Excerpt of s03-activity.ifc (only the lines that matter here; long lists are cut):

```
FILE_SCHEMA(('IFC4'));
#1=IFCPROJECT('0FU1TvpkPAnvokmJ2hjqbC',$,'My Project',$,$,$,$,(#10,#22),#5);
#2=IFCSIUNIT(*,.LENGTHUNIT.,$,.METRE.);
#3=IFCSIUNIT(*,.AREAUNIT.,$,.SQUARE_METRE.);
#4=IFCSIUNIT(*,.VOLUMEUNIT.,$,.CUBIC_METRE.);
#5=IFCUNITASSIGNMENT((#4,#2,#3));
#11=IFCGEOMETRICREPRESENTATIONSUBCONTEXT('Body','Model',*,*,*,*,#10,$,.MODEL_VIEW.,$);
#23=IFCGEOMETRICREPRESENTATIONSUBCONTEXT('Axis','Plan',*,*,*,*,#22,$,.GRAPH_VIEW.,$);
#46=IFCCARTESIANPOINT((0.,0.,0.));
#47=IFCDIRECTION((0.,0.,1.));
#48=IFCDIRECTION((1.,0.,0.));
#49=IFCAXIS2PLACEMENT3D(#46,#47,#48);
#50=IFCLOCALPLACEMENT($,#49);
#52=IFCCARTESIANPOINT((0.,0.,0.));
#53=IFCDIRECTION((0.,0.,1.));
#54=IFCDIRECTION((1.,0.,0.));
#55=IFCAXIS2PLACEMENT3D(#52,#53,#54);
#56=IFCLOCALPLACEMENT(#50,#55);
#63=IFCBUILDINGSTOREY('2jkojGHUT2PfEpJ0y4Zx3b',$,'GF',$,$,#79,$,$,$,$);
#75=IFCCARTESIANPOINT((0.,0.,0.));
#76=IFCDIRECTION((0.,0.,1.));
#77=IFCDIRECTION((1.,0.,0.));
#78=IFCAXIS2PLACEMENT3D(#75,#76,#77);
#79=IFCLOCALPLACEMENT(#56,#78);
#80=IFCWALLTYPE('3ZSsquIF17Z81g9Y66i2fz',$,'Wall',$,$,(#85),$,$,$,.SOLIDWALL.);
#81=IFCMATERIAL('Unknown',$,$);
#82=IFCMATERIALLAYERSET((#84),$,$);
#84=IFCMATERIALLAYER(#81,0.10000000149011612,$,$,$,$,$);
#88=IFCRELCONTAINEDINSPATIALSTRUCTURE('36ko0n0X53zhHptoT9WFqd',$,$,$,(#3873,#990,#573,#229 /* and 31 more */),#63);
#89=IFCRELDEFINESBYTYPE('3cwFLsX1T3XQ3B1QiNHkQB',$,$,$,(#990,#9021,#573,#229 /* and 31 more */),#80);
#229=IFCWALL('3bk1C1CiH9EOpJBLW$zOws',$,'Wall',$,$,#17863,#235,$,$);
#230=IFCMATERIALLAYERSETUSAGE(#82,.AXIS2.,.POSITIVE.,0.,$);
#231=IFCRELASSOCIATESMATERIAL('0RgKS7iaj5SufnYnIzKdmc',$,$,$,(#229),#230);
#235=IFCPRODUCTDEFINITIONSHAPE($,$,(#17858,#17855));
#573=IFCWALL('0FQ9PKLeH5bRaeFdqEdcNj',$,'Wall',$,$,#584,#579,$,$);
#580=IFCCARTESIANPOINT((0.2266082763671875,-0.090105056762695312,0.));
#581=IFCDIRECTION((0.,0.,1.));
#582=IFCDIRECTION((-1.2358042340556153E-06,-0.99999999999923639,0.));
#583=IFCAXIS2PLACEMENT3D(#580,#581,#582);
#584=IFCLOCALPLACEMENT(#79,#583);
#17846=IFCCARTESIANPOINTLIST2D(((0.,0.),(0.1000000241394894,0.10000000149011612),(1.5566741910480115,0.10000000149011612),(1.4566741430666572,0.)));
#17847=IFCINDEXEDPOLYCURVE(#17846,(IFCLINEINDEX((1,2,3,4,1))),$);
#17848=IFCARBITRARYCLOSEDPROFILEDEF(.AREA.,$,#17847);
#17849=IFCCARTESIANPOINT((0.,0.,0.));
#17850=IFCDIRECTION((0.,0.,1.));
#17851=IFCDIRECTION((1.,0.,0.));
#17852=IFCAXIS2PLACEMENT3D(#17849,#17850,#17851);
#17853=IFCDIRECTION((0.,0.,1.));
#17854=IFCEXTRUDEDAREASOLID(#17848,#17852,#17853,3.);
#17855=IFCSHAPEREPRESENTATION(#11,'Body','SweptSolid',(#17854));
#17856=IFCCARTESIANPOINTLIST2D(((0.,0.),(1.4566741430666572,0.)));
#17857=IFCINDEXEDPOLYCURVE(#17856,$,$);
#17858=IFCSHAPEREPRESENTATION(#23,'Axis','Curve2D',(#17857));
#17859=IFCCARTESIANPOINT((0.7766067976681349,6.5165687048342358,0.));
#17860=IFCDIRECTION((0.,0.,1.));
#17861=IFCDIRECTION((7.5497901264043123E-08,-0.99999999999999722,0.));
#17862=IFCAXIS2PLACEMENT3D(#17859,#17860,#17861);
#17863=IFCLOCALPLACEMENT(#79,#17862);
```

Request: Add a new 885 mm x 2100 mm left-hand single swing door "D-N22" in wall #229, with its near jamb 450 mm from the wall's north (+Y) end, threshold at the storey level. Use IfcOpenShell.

```python
import numpy as np
import ifcopenshell
import ifcopenshell.api.feature
import ifcopenshell.api.geometry
import ifcopenshell.api.root
import ifcopenshell.api.spatial
import ifcopenshell.geom
import ifcopenshell.util.element
import ifcopenshell.util.placement
import ifcopenshell.util.representation
import ifcopenshell.util.shape
import ifcopenshell.util.unit

model = ifcopenshell.open("s03-activity.ifc")
unit_scale = ifcopenshell.util.unit.calculate_unit_scale(model)
settings = ifcopenshell.geom.settings()


def volume(element):
    """Net volume in cubic metres, openings subtracted."""
    shape = ifcopenshell.geom.create_shape(settings, element)
    return ifcopenshell.util.shape.get_volume(shape.geometry)


wall = model.by_id(229)
storey = ifcopenshell.util.element.get_container(wall, ifc_class="IfcBuildingStorey")
context = ifcopenshell.util.representation.get_context(model, "Model", "Body", "MODEL_VIEW")
before = volume(wall)

width, height, from_end, sill = 0.885, 2.1, 0.45, 0.0  # metres

# The wall runs along its own X axis, and the end named is its -X end.
wall_shape = ifcopenshell.geom.create_shape(settings, wall)
x, y, z = ifcopenshell.util.shape.get_vertices(wall_shape.geometry).T
start = x.min() + from_end
face, thickness = float(y.min()), float(y.max() - y.min())
wall_matrix = ifcopenshell.util.placement.get_local_placement(wall.ObjectPlacement)
level = ifcopenshell.util.placement.get_local_placement(storey.ObjectPlacement)[2, 3]


def in_wall(x, y):
    """Placement at x, y metres in the wall's axes, at sill height."""
    matrix = wall_matrix.copy()
    matrix[:, 3] = wall_matrix @ np.array([x / unit_scale, y / unit_scale, 0.0, 1.0])
    matrix[2, 3] = level + sill / unit_scale
    return matrix


# Opening: a box that overshoots both wall faces by 50 mm.
opening = ifcopenshell.api.root.create_entity(model, ifc_class="IfcOpeningElement", predefined_type="OPENING")
box = ifcopenshell.api.geometry.add_wall_representation(
    model, context=context, length=width, height=height, thickness=thickness + 0.1
)
ifcopenshell.api.geometry.assign_representation(model, product=opening, representation=box)
ifcopenshell.api.geometry.edit_object_placement(model, product=opening, matrix=in_wall(start, face - 0.05), is_si=False)
ifcopenshell.api.feature.add_feature(model, feature=opening, element=wall)

door = ifcopenshell.api.root.create_entity(model, ifc_class="IfcDoor", name="D-N22", predefined_type="DOOR")
door.OverallWidth, door.OverallHeight = width / unit_scale, height / unit_scale
door.OperationType = "SINGLE_SWING_LEFT"
body = ifcopenshell.api.geometry.add_door_representation(
    model,
    context=context,
    overall_width=door.OverallWidth,
    overall_height=door.OverallHeight,
    operation_type="SINGLE_SWING_LEFT",
    lining_properties={"LiningDepth": thickness / unit_scale, "ThresholdDepth": thickness / unit_scale},
)
ifcopenshell.api.geometry.assign_representation(model, product=door, representation=body)
ifcopenshell.api.spatial.assign_container(model, products=[door], relating_structure=storey)
ifcopenshell.api.feature.add_filling(model, opening=opening, element=door)

# The lining spans the wall, so the door starts at the wall face.
ifcopenshell.api.geometry.edit_object_placement(model, product=door, matrix=in_wall(start, face), is_si=False)

after = volume(wall)

print(f"wall volume {before:.3f} -> {after:.3f} m3")

model.write("s03-activity_rev.ifc")
```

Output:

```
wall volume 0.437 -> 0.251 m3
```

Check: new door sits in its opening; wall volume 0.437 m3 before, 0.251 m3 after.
